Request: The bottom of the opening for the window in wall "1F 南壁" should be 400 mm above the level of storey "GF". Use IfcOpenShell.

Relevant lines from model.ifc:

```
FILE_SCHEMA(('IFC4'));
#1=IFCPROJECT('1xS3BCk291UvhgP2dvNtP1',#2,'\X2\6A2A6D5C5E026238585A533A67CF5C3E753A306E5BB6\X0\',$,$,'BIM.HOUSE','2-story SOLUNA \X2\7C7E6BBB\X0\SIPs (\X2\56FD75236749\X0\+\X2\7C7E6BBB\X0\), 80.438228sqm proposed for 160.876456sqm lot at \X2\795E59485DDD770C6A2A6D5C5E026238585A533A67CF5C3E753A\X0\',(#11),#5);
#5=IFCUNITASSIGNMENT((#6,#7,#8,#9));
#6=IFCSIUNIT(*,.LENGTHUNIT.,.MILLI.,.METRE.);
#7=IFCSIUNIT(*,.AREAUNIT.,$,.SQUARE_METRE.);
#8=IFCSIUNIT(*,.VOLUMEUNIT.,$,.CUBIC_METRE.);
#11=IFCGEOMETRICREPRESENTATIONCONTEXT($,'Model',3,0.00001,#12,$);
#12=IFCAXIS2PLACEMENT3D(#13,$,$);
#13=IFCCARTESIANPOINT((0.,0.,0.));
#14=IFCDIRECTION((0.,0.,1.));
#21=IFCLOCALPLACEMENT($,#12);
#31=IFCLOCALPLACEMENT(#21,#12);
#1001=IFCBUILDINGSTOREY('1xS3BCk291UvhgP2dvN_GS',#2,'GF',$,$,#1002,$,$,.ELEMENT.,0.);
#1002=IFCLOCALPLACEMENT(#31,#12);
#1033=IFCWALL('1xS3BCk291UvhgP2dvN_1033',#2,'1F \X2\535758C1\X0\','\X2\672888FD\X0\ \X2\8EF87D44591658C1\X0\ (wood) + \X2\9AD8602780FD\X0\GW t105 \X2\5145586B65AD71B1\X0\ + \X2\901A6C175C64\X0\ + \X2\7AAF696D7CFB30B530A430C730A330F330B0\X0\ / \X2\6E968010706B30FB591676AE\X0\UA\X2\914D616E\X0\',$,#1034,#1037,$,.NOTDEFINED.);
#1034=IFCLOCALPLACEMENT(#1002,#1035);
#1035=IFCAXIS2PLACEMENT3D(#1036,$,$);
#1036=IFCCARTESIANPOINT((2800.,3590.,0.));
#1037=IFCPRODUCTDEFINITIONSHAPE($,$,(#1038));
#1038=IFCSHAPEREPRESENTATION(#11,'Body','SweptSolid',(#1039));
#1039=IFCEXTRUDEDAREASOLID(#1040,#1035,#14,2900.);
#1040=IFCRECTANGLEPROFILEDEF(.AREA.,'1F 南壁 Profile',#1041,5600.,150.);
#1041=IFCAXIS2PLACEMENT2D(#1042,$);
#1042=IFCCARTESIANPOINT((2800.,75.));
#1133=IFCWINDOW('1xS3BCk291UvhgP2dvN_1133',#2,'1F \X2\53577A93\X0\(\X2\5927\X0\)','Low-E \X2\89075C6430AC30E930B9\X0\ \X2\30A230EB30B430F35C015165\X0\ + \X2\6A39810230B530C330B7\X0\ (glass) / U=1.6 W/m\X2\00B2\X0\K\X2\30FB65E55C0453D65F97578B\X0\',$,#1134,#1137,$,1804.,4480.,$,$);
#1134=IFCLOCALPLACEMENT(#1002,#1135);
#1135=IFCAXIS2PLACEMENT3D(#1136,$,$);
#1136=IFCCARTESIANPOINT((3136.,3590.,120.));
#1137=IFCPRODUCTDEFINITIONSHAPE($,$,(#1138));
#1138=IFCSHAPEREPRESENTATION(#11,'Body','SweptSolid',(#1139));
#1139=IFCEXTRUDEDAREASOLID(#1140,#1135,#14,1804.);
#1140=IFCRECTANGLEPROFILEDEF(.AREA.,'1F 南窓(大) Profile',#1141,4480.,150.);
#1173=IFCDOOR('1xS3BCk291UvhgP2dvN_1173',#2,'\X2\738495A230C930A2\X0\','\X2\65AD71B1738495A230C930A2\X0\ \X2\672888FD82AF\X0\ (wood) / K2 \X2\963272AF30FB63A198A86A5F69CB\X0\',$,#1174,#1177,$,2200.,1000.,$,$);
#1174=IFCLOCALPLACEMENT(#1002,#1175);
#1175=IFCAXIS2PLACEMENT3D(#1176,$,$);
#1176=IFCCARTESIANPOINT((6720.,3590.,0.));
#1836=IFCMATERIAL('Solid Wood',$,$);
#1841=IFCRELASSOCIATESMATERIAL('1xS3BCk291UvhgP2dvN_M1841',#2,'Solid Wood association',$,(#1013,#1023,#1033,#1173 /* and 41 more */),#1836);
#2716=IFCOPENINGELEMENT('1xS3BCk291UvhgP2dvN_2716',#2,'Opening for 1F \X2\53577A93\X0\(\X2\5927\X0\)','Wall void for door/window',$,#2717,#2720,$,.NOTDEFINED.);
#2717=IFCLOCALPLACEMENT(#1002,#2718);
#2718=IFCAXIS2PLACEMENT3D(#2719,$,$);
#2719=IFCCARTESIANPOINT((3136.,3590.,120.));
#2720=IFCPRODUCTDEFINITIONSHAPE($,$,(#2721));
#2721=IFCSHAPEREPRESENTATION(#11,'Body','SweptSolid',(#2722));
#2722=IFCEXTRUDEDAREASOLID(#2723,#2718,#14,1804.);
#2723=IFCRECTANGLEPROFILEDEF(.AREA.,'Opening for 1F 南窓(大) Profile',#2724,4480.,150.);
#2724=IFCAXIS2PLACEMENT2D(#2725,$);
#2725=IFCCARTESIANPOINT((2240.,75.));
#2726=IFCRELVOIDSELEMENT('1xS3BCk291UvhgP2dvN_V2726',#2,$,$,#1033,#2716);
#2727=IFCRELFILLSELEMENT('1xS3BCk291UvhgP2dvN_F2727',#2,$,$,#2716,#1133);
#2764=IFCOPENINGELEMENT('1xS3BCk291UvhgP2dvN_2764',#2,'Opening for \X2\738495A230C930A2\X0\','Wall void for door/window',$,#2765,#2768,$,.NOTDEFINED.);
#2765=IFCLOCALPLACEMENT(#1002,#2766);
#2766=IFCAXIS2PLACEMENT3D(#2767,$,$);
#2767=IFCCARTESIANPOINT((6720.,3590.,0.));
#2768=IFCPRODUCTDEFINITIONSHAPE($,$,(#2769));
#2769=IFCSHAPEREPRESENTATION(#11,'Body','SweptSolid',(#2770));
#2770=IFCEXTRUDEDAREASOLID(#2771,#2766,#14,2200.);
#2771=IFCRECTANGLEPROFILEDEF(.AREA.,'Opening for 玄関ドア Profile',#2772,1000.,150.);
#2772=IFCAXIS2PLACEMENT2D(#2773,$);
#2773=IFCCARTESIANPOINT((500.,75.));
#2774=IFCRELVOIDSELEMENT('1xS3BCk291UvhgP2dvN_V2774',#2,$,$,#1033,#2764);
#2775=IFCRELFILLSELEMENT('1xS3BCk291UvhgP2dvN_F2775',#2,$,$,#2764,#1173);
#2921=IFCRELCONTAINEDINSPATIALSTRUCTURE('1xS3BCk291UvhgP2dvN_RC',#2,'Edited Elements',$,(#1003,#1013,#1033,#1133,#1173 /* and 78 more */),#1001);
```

```python
import numpy as np
import ifcopenshell
import ifcopenshell.api.geometry
import ifcopenshell.geom
import ifcopenshell.util.element
import ifcopenshell.util.placement
import ifcopenshell.util.shape
import ifcopenshell.util.unit

model = ifcopenshell.open("model.ifc")
unit_scale = ifcopenshell.util.unit.calculate_unit_scale(model)

window = model.by_guid("1xS3BCk291UvhgP2dvN_1133")
opening = window.FillsVoids[0].RelatingOpeningElement
storey = ifcopenshell.util.element.get_container(window, ifc_class="IfcBuildingStorey")
level = ifcopenshell.util.placement.get_local_placement(storey.ObjectPlacement)[2, 3]

# The opening's origin need not be at the sill, so measure its lowest point.
shape = ifcopenshell.geom.create_shape(ifcopenshell.geom.settings(), opening)
bottom = ifcopenshell.util.shape.get_shape_bottom_elevation(shape, shape.geometry) / unit_scale
dz = level + 0.4 / unit_scale - bottom

shift = np.array([0.0, 0.0, dz])
# The window is not placed relative to its opening, so move both.
for product in (opening, window):
    matrix = ifcopenshell.util.placement.get_local_placement(product.ObjectPlacement)
    matrix[:3, 3] += shift
    ifcopenshell.api.geometry.edit_object_placement(model, product=product, matrix=matrix, is_si=False)

print(f"moved by {dz * unit_scale:+.3f} m")

model.write("model_edited.ifc")
```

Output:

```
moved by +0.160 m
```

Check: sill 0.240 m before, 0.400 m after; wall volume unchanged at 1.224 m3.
